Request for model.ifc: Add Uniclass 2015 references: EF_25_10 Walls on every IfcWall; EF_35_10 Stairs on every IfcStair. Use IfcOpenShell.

First a look at what the model holds.

```python
import ifcopenshell

model = ifcopenshell.open("model.ifc")
print(model.schema)
print("classifications:", [c.Name for c in model.by_type("IfcClassification")])
for ifc_class in ("IfcDoor", "IfcRoof", "IfcStair", "IfcWall", "IfcWindow"):
    print(ifc_class, len(model.by_type(ifc_class)))
```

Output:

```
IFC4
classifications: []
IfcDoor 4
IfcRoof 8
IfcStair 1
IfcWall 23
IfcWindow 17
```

```python
import ifcopenshell
import ifcopenshell.api.classification

model = ifcopenshell.open("model.ifc")

system = ifcopenshell.api.classification.add_classification(model, classification="Uniclass 2015")

codes = {
    "IfcWall": ("EF_25_10", "Walls"),
    "IfcStair": ("EF_35_10", "Stairs"),
}
for ifc_class, (code, name) in codes.items():
    products = model.by_type(ifc_class)
    ifcopenshell.api.classification.add_reference(
        model, products=products, classification=system, identification=code, name=name
    )
    print(code, len(products))

model.write("model_edited.ifc")
```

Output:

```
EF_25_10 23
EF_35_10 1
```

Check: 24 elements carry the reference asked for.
